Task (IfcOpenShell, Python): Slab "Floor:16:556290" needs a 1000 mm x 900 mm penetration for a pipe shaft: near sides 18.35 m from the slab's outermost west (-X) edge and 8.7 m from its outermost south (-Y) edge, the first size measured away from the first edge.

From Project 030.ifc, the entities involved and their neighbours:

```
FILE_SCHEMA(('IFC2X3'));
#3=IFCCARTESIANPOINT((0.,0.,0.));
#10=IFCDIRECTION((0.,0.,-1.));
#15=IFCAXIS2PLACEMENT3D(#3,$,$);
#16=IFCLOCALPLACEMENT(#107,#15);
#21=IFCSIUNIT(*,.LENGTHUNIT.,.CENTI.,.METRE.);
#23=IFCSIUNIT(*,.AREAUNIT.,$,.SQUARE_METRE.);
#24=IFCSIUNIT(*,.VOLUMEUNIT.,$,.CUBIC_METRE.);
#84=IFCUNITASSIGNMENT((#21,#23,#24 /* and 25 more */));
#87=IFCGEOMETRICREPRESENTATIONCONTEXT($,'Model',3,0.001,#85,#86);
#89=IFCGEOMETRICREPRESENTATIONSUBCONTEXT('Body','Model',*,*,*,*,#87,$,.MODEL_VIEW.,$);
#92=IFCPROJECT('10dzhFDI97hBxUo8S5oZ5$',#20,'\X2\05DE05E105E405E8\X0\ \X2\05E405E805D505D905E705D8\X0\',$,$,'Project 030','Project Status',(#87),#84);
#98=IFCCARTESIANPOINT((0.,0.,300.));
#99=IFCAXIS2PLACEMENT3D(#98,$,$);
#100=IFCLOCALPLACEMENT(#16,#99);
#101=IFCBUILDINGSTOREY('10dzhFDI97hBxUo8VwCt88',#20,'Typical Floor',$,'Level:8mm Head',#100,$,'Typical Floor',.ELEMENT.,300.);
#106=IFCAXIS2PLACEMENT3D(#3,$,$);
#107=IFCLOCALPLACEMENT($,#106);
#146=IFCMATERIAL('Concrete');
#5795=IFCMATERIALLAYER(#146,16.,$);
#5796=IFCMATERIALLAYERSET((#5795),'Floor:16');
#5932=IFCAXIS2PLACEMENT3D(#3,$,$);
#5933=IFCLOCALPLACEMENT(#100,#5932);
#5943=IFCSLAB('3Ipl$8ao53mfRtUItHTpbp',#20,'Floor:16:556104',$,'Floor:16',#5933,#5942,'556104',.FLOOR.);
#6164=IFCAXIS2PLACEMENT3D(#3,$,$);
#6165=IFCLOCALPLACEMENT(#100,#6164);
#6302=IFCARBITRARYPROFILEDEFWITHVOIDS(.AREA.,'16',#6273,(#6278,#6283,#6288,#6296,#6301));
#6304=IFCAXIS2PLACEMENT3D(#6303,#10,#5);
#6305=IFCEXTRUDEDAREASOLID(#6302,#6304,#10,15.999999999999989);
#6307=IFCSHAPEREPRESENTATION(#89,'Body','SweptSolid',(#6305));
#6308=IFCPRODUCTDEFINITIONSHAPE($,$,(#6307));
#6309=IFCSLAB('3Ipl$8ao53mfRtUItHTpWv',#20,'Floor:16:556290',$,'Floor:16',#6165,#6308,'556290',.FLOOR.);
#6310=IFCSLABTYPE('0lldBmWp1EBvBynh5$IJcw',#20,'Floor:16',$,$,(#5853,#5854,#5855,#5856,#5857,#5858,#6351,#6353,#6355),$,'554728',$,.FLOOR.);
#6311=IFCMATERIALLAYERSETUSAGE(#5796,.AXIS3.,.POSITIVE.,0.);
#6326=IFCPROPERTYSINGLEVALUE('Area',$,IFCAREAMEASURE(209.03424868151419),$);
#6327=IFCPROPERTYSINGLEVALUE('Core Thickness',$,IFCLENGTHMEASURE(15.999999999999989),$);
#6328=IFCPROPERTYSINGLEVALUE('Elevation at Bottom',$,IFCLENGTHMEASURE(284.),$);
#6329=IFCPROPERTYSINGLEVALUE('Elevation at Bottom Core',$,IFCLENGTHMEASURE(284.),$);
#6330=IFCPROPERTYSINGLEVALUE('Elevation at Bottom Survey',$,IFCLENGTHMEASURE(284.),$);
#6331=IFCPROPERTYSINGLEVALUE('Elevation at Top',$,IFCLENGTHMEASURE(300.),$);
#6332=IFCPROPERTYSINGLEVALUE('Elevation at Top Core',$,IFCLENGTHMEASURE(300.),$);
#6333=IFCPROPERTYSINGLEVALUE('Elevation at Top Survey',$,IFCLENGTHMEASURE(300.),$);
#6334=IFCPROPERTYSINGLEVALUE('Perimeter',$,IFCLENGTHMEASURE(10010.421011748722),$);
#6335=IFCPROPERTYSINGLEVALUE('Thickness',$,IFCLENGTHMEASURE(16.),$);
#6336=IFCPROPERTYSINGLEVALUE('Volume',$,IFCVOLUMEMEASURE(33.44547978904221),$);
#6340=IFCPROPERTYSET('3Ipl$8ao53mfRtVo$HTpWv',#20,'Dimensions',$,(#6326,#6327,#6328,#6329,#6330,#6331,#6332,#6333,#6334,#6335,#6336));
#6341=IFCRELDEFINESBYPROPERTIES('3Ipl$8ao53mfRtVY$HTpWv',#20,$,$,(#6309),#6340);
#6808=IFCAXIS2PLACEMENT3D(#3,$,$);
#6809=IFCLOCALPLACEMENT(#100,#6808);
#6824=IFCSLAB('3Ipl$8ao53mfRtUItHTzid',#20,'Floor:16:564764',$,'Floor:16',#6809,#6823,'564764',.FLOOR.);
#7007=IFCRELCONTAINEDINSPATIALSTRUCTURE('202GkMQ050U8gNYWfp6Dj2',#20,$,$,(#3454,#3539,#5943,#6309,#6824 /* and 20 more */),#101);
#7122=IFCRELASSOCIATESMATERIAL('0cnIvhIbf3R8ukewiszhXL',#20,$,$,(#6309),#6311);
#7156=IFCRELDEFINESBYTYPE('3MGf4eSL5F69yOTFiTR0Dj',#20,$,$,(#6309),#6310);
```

```python
import numpy as np
import ifcopenshell
import ifcopenshell.api.feature
import ifcopenshell.api.geometry
import ifcopenshell.api.pset
import ifcopenshell.api.root
import ifcopenshell.geom
import ifcopenshell.util.element
import ifcopenshell.util.placement
import ifcopenshell.util.representation
import ifcopenshell.util.shape
import ifcopenshell.util.unit

model = ifcopenshell.open("Project 030.ifc")
unit_scale = ifcopenshell.util.unit.calculate_unit_scale(model)
area_scale = ifcopenshell.util.unit.calculate_unit_scale(model, "AREAUNIT")
volume_scale = ifcopenshell.util.unit.calculate_unit_scale(model, "VOLUMEUNIT")
settings = ifcopenshell.geom.settings()


def volume(element):
    """Net volume in cubic metres, openings subtracted."""
    shape = ifcopenshell.geom.create_shape(settings, element)
    return ifcopenshell.util.shape.get_volume(shape.geometry)


slab = model.by_id(6309)
before = volume(slab)

# Extent in the slab's own axes, in metres. The edges named are its -X and -Y sides.
slab_shape = ifcopenshell.geom.create_shape(settings, slab)
vertices = ifcopenshell.util.shape.get_vertices(slab_shape.geometry)
x_min, y_min, bottom = vertices.min(axis=0)
top = vertices[:, 2].max()

opening = ifcopenshell.api.root.create_entity(model, ifc_class="IfcOpeningElement", name="Pipe shaft opening")
context = ifcopenshell.util.representation.get_context(model, "Model", "Body", "MODEL_VIEW")
width, depth = 1, 0.9
outline = [(0.0, 0.0), (width, 0.0), (width, depth), (0.0, depth), (0.0, 0.0)]
# Overshoot both faces by 50 mm so the cut is clean.
shape = ifcopenshell.api.geometry.add_slab_representation(
    model, context=context, depth=top - bottom + 0.1, polyline=outline
)
ifcopenshell.api.geometry.assign_representation(model, product=opening, representation=shape)

matrix = ifcopenshell.util.placement.get_local_placement(slab.ObjectPlacement)
matrix[:, 3] = matrix @ np.append(np.array([x_min + 18.35, y_min + 8.7, bottom - 0.05]) / unit_scale, 1.0)
ifcopenshell.api.geometry.edit_object_placement(model, product=opening, matrix=matrix, is_si=False)
ifcopenshell.api.feature.add_feature(model, feature=opening, element=slab)

after = volume(slab)

# Update the slab's stored quantities.
pset = model.by_id(ifcopenshell.util.element.get_pset(slab, "Dimensions", should_inherit=False)["id"])
ifcopenshell.api.pset.edit_pset(model, pset=pset, properties={
    "Area": model.create_entity("IfcAreaMeasure", after / (top - bottom) / area_scale),
    "Volume": model.create_entity("IfcVolumeMeasure", after / volume_scale),
})

print(f"slab volume {before:.3f} -> {after:.3f} m3")

model.write("Project 030_edited.ifc")
```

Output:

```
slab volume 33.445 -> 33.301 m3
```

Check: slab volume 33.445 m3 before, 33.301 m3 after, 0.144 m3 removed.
